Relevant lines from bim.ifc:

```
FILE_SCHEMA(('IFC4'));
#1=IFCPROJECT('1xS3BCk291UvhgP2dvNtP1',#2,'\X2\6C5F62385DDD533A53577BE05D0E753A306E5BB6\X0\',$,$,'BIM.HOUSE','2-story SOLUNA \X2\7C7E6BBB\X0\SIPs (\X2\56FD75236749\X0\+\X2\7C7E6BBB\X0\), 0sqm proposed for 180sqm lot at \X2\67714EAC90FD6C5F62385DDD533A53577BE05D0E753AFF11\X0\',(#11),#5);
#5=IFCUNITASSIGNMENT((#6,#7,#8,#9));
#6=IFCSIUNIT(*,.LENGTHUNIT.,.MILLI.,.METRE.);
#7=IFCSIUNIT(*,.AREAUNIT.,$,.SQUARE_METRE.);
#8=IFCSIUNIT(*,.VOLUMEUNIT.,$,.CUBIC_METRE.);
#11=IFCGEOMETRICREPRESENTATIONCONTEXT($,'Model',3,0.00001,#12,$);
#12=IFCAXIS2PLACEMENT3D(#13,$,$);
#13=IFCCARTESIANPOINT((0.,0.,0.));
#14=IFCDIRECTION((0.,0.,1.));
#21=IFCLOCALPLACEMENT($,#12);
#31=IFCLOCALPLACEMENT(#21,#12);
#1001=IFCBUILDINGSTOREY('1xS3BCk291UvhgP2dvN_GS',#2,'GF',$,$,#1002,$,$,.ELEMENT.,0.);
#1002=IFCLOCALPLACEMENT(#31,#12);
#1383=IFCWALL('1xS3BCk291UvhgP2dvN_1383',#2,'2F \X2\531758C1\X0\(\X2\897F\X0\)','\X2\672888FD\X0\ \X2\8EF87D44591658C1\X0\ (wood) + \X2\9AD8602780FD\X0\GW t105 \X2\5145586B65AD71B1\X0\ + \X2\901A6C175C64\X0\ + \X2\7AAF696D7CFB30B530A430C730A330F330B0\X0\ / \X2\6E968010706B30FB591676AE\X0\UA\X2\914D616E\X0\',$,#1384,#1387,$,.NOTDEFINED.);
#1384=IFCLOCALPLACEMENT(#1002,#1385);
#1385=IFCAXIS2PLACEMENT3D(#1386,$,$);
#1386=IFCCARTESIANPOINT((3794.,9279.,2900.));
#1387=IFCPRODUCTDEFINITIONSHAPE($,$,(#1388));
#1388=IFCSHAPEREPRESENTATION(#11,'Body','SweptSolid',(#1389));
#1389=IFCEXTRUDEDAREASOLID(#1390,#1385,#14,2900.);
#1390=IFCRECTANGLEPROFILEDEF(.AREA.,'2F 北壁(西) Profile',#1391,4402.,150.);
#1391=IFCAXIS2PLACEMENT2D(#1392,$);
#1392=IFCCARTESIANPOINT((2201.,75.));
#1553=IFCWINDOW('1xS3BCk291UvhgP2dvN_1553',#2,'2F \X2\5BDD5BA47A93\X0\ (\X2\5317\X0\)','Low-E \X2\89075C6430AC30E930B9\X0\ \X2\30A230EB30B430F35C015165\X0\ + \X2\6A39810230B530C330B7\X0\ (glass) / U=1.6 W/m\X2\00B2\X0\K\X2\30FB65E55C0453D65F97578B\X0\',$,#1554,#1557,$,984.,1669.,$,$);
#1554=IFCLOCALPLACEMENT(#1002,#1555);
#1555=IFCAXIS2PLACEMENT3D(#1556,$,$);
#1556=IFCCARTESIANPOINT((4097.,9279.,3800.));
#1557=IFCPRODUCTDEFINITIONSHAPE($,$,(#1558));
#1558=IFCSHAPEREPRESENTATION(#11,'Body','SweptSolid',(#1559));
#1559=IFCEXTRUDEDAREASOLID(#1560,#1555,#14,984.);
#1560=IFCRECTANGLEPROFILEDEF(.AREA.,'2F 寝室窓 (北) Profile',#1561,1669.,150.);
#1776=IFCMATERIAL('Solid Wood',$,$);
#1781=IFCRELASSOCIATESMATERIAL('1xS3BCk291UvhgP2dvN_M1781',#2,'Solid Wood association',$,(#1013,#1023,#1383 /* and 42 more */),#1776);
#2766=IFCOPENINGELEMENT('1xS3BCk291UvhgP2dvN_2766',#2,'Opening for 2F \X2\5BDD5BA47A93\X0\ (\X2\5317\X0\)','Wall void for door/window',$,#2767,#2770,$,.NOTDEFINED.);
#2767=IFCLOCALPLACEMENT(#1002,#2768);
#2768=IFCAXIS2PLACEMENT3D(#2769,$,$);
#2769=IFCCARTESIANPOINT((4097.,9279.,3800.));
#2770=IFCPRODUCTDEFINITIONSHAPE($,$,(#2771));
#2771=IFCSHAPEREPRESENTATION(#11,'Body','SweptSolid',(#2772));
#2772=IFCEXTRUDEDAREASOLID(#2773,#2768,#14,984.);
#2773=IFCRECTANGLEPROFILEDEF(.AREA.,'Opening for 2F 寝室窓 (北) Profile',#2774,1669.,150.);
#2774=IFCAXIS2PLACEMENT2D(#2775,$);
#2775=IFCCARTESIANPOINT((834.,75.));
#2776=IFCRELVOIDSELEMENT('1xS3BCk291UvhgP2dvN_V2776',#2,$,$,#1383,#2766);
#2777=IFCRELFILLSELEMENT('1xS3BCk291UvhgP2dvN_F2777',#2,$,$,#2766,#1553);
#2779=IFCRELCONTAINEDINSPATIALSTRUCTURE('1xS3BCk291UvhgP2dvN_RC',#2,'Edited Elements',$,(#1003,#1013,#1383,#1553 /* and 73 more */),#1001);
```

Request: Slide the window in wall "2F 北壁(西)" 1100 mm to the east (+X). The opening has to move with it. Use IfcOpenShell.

```python
import ifcopenshell
import ifcopenshell.api.geometry
import ifcopenshell.util.placement

model = ifcopenshell.open("bim.ifc")

window = model.by_id(1553)
opening = window.FillsVoids[0].RelatingOpeningElement
wall = opening.VoidsElements[0].RelatingBuildingElement

wall_matrix = ifcopenshell.util.placement.get_local_placement(wall.ObjectPlacement)
shift = wall_matrix[:3, 0] * 1100.0
before = ifcopenshell.util.placement.get_local_placement(window.ObjectPlacement)[:3, 3].copy()

# The window is not placed relative to its opening, so move both.
for product in (opening, window):
    matrix = ifcopenshell.util.placement.get_local_placement(product.ObjectPlacement)
    matrix[:3, 3] += shift
    ifcopenshell.api.geometry.edit_object_placement(model, product=product, matrix=matrix, is_si=False)

after = ifcopenshell.util.placement.get_local_placement(window.ObjectPlacement)[:3, 3]
print("window moved by", (after - before).round(3) + 0.0)

model.write("bim_rev.ifc")
```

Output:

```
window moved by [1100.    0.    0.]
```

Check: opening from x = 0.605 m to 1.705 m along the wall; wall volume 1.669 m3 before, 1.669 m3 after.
